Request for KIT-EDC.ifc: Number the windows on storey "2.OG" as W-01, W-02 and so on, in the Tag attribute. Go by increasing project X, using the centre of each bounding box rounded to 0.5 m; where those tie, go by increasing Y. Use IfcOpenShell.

First a look at what the model holds.

```python
import ifcopenshell
import ifcopenshell.util.element
import ifcopenshell.util.placement

model = ifcopenshell.open("KIT-EDC.ifc")
print(model.schema)
storey = next(s for s in model.by_type("IfcBuildingStorey") if s.Name == "2.OG")
windows = [e for e in ifcopenshell.util.element.get_decomposition(storey) if e.is_a("IfcWindow")]
for e in sorted(windows, key=lambda e: e.id()):
    origin = ifcopenshell.util.placement.get_local_placement(e.ObjectPlacement)[:3, 3]
    print(e.id(), e.Tag, e.Name, origin.round(2) + 0.0, sep=" | ")
```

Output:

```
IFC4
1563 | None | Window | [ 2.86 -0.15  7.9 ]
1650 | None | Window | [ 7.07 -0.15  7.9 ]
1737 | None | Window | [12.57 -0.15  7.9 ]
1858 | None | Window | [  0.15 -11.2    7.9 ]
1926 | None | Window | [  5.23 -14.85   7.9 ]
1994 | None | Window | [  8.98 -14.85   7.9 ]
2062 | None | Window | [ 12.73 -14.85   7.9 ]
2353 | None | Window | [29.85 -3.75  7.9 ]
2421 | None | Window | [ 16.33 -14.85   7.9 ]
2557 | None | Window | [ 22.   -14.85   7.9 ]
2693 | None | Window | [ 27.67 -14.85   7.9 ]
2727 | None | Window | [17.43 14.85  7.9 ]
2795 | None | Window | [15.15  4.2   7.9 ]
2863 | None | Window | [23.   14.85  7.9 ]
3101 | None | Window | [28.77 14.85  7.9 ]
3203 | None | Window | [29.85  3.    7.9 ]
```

```python
import ifcopenshell
import ifcopenshell.geom
import ifcopenshell.util.element
import ifcopenshell.util.shape

model = ifcopenshell.open("KIT-EDC.ifc")
settings = ifcopenshell.geom.settings()
settings.set("use-world-coords", True)


def centre(element):
    shape = ifcopenshell.geom.create_shape(settings, element)
    return ifcopenshell.util.shape.get_bbox_centroid(shape.geometry)


storey = next(s for s in model.by_type("IfcBuildingStorey") if s.Name == "2.OG")
windows = [e for e in ifcopenshell.util.element.get_decomposition(storey) if e.is_a("IfcWindow")]

# Insertion points can sit at a corner or the storey origin, so sort by the geometry (in metres).
centres = {e: centre(e) for e in windows}
windows.sort(key=lambda e: (round(centres[e][0] / 0.5), centres[e][1]))

for i, e in enumerate(windows, start=1):
    number = f"W-{i:02d}"
    e.Tag = number
    print(e.id(), number)

model.write("KIT-EDC_v2.ifc")
```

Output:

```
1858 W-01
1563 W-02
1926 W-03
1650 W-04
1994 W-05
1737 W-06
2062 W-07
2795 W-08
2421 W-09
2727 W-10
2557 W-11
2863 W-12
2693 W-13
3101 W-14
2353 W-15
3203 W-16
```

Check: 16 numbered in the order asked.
